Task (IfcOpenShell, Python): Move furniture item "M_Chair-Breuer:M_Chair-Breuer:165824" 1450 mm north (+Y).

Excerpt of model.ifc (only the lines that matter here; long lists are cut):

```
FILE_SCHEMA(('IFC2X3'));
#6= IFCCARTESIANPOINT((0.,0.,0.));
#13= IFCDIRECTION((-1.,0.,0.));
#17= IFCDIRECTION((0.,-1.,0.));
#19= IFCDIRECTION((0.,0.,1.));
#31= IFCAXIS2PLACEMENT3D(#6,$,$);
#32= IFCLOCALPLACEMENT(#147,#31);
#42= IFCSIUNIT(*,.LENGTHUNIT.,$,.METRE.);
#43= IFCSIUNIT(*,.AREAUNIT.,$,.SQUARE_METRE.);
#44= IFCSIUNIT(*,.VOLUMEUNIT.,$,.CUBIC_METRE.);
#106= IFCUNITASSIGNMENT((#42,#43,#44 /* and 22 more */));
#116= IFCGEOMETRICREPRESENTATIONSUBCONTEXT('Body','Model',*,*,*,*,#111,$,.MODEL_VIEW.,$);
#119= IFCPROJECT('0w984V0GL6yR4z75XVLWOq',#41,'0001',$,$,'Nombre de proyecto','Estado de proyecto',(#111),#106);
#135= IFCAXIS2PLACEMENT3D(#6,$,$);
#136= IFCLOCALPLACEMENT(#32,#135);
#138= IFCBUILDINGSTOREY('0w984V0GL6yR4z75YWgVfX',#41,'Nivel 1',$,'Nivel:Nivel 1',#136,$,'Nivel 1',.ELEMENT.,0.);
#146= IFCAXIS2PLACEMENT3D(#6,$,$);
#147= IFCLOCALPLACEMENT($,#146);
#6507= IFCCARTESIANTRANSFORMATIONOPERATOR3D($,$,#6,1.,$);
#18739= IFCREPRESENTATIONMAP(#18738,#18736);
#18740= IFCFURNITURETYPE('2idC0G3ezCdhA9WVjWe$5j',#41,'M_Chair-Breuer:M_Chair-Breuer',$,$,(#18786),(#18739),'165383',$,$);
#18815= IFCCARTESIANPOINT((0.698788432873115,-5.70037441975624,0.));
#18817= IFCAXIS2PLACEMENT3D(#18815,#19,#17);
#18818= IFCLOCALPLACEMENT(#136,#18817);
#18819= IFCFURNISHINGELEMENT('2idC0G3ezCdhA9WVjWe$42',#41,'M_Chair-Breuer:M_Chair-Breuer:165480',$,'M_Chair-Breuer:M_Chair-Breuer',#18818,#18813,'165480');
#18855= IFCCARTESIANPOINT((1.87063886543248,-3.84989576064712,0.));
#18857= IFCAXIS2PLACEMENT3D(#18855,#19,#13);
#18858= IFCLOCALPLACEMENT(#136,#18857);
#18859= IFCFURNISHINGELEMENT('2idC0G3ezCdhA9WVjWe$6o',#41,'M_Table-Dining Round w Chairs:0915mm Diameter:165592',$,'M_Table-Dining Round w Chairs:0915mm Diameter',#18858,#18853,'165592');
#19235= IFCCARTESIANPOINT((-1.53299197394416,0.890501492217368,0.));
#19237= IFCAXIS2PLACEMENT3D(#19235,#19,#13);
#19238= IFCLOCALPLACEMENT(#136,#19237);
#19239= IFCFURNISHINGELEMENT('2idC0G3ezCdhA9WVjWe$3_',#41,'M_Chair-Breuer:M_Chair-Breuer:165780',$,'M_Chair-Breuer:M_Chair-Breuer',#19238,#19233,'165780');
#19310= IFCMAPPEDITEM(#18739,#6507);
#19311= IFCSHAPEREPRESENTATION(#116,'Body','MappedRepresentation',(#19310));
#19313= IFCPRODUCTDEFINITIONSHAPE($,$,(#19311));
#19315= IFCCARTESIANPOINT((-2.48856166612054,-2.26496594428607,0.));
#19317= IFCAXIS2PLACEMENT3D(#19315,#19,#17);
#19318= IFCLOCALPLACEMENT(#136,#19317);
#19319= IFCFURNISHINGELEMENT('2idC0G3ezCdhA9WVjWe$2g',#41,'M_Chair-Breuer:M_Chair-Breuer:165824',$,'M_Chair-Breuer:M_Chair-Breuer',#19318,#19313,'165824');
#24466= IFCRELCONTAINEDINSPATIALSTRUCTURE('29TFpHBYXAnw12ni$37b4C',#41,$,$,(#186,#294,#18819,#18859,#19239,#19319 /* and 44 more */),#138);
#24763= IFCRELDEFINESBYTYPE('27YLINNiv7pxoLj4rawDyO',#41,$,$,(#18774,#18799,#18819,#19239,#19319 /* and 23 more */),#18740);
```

```python
import ifcopenshell
import ifcopenshell.api.geometry
import ifcopenshell.util.placement

model = ifcopenshell.open("model.ifc")

item = model.by_id(19319)
matrix = ifcopenshell.util.placement.get_local_placement(item.ObjectPlacement)
matrix[1, 3] += 1.45
ifcopenshell.api.geometry.edit_object_placement(model, product=item, matrix=matrix, is_si=False)

print(ifcopenshell.util.placement.get_local_placement(item.ObjectPlacement).round(3) + 0.0)

model.write("model_rev.ifc")
```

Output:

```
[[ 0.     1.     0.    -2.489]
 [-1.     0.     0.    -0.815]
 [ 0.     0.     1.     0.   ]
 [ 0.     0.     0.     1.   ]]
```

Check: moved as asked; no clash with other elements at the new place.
